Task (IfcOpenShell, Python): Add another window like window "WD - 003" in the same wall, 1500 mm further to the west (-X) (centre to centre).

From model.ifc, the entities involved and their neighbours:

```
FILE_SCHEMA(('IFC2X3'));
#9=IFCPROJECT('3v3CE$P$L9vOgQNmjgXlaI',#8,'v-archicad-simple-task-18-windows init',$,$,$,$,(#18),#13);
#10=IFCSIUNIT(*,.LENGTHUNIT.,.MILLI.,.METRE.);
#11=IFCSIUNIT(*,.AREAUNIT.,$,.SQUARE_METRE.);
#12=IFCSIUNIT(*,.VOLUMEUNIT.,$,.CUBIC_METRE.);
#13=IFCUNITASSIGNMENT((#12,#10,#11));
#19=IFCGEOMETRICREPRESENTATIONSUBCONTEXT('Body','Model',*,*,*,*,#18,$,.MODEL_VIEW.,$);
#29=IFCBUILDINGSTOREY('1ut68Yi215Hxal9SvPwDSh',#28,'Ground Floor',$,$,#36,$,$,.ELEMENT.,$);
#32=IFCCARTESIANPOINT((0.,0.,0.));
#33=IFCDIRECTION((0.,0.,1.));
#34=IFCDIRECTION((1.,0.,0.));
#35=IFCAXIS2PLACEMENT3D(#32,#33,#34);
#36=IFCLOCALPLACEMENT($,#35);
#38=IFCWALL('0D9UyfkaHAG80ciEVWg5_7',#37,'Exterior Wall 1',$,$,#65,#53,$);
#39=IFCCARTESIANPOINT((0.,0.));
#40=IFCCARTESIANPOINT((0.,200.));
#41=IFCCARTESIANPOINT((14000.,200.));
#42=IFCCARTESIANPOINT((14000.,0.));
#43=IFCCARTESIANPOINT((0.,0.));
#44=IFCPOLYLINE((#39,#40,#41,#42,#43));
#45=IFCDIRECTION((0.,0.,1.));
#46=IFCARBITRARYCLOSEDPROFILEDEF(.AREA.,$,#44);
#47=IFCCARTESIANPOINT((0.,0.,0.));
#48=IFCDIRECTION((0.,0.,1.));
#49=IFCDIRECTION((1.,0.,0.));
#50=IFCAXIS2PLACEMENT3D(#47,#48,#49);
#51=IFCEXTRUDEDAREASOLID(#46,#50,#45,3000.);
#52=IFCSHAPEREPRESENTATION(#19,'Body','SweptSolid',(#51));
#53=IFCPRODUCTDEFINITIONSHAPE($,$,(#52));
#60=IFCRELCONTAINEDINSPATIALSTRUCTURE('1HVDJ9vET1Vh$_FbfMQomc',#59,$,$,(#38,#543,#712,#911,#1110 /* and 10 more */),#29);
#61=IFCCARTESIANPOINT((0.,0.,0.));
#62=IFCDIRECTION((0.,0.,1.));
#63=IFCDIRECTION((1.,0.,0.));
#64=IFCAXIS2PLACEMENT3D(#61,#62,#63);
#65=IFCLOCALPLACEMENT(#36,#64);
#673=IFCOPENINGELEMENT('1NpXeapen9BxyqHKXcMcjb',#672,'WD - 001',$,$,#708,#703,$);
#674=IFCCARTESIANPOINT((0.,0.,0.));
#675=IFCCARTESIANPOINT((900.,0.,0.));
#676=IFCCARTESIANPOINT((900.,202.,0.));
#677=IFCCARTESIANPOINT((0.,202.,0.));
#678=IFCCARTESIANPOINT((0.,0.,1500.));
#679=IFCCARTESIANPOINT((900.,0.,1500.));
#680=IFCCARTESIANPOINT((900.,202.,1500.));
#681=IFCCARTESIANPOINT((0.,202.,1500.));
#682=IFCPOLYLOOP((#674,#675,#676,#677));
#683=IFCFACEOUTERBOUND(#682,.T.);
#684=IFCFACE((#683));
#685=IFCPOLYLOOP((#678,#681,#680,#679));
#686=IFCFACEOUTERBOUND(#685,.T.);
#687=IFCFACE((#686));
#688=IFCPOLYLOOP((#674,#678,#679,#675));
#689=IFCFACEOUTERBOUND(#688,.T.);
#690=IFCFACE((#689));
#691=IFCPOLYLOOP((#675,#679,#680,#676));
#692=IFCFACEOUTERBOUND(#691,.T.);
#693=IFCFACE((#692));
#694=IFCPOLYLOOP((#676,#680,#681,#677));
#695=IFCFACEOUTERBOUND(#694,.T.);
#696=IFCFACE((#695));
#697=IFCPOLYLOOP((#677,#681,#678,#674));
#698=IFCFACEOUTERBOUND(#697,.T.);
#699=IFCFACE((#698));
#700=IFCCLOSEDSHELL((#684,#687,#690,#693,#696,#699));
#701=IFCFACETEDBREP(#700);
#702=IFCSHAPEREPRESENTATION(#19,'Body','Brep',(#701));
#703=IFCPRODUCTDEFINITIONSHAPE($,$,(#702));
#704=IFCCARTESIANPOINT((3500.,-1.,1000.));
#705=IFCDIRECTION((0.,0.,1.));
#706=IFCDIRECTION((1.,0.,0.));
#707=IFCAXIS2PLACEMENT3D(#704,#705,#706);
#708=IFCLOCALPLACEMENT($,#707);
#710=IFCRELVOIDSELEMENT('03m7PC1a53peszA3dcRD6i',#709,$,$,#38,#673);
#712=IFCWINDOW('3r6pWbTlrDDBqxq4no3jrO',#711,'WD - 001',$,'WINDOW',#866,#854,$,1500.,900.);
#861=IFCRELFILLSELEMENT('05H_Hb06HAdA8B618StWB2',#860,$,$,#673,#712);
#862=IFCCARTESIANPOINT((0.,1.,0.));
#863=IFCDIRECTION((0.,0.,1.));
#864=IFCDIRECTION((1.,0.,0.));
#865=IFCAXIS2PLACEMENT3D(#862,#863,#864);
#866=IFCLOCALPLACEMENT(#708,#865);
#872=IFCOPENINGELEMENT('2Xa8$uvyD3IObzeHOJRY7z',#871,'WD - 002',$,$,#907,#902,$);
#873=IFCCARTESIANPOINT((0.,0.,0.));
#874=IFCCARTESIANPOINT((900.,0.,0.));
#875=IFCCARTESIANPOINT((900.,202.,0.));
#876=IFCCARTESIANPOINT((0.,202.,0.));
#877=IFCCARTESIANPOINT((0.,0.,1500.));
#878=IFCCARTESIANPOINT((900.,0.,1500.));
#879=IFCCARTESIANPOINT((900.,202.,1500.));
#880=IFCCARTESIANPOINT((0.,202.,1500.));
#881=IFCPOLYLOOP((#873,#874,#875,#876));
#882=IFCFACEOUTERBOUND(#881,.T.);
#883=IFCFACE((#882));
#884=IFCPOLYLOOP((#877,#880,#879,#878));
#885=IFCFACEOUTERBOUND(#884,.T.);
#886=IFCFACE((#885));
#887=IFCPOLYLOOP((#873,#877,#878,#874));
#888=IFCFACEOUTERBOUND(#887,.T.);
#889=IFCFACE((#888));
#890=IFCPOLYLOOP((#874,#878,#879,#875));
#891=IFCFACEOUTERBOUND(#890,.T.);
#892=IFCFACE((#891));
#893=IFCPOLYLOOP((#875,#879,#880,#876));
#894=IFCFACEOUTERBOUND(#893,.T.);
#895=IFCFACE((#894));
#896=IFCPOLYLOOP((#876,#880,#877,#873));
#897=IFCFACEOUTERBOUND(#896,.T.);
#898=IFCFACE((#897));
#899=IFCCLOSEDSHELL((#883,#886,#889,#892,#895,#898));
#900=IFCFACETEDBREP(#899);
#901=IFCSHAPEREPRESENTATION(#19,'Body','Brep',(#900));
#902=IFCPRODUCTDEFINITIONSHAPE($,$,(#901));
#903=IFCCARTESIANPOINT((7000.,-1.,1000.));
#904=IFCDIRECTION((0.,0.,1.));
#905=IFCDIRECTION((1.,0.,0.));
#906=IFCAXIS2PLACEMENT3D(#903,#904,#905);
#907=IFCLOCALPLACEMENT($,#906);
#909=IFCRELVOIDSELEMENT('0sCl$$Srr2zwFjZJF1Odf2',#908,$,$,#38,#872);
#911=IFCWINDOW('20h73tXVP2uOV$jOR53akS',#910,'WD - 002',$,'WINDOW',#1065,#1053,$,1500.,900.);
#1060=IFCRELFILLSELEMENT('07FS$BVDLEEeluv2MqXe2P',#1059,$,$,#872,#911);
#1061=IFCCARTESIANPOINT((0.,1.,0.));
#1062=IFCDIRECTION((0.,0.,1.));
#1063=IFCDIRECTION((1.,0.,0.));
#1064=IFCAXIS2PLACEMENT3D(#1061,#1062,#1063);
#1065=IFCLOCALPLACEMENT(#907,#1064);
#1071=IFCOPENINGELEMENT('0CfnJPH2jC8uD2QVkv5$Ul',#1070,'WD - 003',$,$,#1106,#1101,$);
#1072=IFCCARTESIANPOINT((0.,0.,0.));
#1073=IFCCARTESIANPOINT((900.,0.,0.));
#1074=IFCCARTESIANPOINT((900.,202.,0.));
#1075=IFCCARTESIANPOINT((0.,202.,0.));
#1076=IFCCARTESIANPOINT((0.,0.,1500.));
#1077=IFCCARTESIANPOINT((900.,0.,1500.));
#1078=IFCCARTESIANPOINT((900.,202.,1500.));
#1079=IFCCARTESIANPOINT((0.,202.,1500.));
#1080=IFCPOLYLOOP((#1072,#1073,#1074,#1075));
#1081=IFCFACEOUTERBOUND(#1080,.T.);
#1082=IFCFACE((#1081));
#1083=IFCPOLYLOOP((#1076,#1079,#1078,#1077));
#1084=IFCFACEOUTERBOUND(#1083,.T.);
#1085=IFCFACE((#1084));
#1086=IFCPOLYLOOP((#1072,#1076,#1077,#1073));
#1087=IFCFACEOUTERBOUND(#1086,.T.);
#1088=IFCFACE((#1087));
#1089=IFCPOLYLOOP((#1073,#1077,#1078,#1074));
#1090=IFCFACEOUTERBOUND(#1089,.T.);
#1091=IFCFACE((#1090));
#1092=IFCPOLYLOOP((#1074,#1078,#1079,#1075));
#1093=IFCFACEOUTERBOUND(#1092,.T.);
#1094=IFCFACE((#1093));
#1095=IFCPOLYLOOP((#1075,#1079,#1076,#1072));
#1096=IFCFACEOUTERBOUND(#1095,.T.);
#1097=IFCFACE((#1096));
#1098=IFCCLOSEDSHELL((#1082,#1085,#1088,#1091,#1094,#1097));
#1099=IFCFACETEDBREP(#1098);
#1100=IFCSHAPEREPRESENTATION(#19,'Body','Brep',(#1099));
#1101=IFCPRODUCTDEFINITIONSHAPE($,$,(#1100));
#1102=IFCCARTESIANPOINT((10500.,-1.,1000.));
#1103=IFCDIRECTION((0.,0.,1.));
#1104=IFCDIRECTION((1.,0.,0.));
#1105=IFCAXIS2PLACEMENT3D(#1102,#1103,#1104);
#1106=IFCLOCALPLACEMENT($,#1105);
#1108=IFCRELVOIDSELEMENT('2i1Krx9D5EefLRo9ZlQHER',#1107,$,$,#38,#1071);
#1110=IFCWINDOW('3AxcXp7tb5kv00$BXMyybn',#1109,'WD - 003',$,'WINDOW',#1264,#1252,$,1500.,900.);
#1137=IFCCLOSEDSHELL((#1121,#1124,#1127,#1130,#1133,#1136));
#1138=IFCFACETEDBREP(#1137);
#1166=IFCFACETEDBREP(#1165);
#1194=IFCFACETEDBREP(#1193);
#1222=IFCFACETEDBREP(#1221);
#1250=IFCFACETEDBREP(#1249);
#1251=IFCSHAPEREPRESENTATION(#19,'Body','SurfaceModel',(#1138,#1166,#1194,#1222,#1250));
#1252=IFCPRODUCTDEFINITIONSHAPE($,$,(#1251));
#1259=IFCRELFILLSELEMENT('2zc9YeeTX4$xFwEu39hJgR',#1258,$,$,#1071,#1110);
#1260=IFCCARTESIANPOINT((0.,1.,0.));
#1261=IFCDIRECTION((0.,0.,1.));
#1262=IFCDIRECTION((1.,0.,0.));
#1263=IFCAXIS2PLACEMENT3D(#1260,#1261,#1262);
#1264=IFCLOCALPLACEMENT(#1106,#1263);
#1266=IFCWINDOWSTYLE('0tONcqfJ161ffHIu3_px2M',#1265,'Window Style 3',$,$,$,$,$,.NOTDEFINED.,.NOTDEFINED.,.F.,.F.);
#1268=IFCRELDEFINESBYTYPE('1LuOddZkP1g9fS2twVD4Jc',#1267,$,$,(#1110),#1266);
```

```python
import ifcopenshell
import ifcopenshell.api.feature
import ifcopenshell.api.geometry
import ifcopenshell.api.root
import ifcopenshell.geom
import ifcopenshell.util.element
import ifcopenshell.util.placement
import ifcopenshell.util.shape
import ifcopenshell.util.unit

model = ifcopenshell.open("model.ifc")
unit_scale = ifcopenshell.util.unit.calculate_unit_scale(model)
settings = ifcopenshell.geom.settings()


def volume(element):
    """Net volume in cubic metres, openings subtracted."""
    shape = ifcopenshell.geom.create_shape(settings, element)
    return ifcopenshell.util.shape.get_volume(shape.geometry)


window = model.by_id(1110)
opening = window.FillsVoids[0].RelatingOpeningElement
wall = opening.VoidsElements[0].RelatingBuildingElement
before = volume(wall)
shift = ifcopenshell.util.placement.get_local_placement(wall.ObjectPlacement)[:3, 0] * -1.5 / unit_scale

# copy_class copies the void relationship, type, container and properties, but no geometry.
new_opening = ifcopenshell.api.root.copy_class(model, product=opening)
new_opening.Representation = ifcopenshell.util.element.copy_deep(
    model, opening.Representation, exclude=["IfcGeometricRepresentationContext", "IfcRepresentationMap"]
)
new_window = ifcopenshell.api.root.copy_class(model, product=window)
new_window.Representation = ifcopenshell.util.element.copy_deep(
    model, window.Representation, exclude=["IfcGeometricRepresentationContext", "IfcRepresentationMap"]
)
fills = ifcopenshell.api.feature.add_filling(model, opening=new_opening, element=new_window)
fills.OwnerHistory = new_window.OwnerHistory  # required in IFC2X3

for old, new in ((opening, new_opening), (window, new_window)):
    matrix = ifcopenshell.util.placement.get_local_placement(old.ObjectPlacement)
    matrix[:3, 3] += shift
    ifcopenshell.api.geometry.edit_object_placement(model, product=new, matrix=matrix, is_si=False)

after = volume(wall)

print(f"wall volume {before:.3f} -> {after:.3f} m3")

model.write("model_rev.ifc")
```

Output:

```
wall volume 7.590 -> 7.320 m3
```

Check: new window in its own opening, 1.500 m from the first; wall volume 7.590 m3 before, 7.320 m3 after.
